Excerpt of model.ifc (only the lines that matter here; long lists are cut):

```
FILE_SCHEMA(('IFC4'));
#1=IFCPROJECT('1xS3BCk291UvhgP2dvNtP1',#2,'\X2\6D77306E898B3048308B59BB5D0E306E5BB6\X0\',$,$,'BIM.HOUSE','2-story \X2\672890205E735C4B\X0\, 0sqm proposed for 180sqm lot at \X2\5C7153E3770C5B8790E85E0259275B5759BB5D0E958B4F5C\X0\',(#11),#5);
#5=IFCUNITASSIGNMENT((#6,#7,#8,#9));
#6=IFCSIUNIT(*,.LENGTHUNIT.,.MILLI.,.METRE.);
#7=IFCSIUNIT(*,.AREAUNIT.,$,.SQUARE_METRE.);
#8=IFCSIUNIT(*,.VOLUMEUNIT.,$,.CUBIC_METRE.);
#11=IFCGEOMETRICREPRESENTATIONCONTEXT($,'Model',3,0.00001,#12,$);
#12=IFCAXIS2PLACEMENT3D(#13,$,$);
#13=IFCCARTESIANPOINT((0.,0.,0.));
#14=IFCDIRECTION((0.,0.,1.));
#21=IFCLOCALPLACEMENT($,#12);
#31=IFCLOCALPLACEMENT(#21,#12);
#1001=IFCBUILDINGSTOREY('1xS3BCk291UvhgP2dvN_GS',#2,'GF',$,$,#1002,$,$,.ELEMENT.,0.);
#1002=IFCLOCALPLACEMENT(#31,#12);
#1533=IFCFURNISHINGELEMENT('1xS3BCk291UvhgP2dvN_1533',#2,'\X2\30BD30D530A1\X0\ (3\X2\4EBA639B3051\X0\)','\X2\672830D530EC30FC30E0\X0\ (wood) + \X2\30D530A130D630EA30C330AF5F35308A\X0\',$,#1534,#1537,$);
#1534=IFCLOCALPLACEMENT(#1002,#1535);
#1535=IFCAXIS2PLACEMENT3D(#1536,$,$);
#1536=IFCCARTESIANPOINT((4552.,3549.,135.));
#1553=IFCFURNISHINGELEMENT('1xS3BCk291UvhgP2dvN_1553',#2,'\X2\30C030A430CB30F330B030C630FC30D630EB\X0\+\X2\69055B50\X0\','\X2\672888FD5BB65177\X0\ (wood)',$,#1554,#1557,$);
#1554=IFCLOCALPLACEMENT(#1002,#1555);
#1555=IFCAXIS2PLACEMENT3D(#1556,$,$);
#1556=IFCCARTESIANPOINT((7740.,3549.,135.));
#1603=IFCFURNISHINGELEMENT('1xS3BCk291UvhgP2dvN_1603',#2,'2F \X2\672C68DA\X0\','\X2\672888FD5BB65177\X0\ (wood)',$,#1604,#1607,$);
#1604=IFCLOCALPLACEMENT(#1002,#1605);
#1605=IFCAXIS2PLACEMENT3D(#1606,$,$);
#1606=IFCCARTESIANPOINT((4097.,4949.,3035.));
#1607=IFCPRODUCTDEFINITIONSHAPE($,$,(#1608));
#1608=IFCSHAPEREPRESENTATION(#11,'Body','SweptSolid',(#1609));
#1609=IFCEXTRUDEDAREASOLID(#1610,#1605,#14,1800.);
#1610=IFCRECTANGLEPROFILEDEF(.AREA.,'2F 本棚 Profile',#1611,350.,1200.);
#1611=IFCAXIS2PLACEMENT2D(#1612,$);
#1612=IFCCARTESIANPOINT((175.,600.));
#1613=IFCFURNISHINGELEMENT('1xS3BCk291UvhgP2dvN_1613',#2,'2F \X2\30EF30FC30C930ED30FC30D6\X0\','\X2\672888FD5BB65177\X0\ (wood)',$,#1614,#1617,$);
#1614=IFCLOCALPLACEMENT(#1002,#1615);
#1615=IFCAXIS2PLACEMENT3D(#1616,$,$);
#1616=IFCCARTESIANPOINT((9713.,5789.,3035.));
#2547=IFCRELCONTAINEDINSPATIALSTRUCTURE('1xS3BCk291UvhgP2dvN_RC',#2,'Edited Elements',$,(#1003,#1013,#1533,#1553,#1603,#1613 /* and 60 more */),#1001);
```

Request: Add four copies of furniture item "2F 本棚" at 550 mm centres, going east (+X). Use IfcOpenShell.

```python
import numpy as np
import ifcopenshell
import ifcopenshell.api.geometry
import ifcopenshell.api.root
import ifcopenshell.util.element
import ifcopenshell.util.placement
import ifcopenshell.util.unit

model = ifcopenshell.open("model.ifc")
unit_scale = ifcopenshell.util.unit.calculate_unit_scale(model)


def reuse_history(source, copy):
    """copy_class also copies each property set's owner history, people and application; keep the originals."""
    for rel in copy.IsDefinedBy:
        if rel.is_a("IfcRelDefinesByProperties") and (history := rel.RelatingPropertyDefinition.OwnerHistory):
            rel.RelatingPropertyDefinition.OwnerHistory = source.OwnerHistory
            ifcopenshell.util.element.remove_deep2(model, history)


source = model.by_guid("1xS3BCk291UvhgP2dvN_1603")
base = ifcopenshell.util.placement.get_local_placement(source.ObjectPlacement)
step = np.array([1.0, 0.0, 0.0]) * 0.55 / unit_scale

for i in range(1, 5):
    copy = ifcopenshell.api.root.copy_class(model, product=source)
    copy.Representation = ifcopenshell.util.element.copy_deep(
        model, source.Representation, exclude=["IfcGeometricRepresentationContext", "IfcRepresentationMap"]
    )
    reuse_history(source, copy)
    matrix = base.copy()
    matrix[:3, 3] += i * step
    print("added at", matrix[:3, 3].round(3) + 0.0)
    ifcopenshell.api.geometry.edit_object_placement(model, product=copy, matrix=matrix, is_si=False)

model.write("model_edited.ifc")
```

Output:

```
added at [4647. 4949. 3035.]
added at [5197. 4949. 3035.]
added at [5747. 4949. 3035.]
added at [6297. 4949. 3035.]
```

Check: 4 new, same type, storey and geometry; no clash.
